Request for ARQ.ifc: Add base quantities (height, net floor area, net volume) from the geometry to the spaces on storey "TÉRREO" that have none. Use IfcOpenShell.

First a look at what the model holds.

```python
import ifcopenshell
import ifcopenshell.util.element
import ifcopenshell.util.unit

model = ifcopenshell.open("ARQ.ifc")
print(model.schema)
for unit_type in ("LENGTHUNIT", "AREAUNIT", "VOLUMEUNIT"):
    print(unit_type, ifcopenshell.util.unit.calculate_unit_scale(model, unit_type))
storey = next(s for s in model.by_type("IfcBuildingStorey") if s.Name == "TÉRREO")
spaces = [e for e in ifcopenshell.util.element.get_decomposition(storey) if e.is_a("IfcSpace")]
for e in sorted(spaces, key=lambda e: e.id()):
    print(e.id(), e.is_a(), e.Name, list(ifcopenshell.util.element.get_psets(e, qtos_only=True)), sep=" | ")
```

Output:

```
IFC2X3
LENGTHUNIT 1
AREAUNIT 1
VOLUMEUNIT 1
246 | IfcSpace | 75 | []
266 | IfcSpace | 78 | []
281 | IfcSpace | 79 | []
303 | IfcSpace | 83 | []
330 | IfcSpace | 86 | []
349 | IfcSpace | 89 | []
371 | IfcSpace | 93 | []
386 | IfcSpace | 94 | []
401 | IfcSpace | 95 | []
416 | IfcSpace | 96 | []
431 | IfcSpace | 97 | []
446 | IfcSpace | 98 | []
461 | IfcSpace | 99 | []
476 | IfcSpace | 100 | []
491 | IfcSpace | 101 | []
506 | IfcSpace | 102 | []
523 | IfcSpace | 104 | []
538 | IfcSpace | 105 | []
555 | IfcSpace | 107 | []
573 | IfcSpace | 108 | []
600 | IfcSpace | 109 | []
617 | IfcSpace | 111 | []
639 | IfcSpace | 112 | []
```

```python
import ifcopenshell
import ifcopenshell.api.pset
import ifcopenshell.geom
import ifcopenshell.util.element
import ifcopenshell.util.shape
import ifcopenshell.util.unit

model = ifcopenshell.open("ARQ.ifc")
unit_scale = ifcopenshell.util.unit.calculate_unit_scale(model)
area_scale = ifcopenshell.util.unit.calculate_unit_scale(model, "AREAUNIT")
volume_scale = ifcopenshell.util.unit.calculate_unit_scale(model, "VOLUMEUNIT")
settings = ifcopenshell.geom.settings()

storey = next(s for s in model.by_type("IfcBuildingStorey") if s.Name == "TÉRREO")
spaces = [e for e in ifcopenshell.util.element.get_decomposition(storey) if e.is_a("IfcSpace")]

for e in sorted(spaces, key=lambda e: e.id()):
    if ifcopenshell.util.element.get_psets(e, qtos_only=True, should_inherit=False):
        continue
    # Geometry comes back in metres, in the element's own axes.
    shape = ifcopenshell.geom.create_shape(settings, e)
    values = {
        "Height": ifcopenshell.util.shape.get_z(shape.geometry) / unit_scale,
        "NetFloorArea": ifcopenshell.util.shape.get_footprint_area(shape.geometry) / area_scale,
        "NetVolume": ifcopenshell.util.shape.get_volume(shape.geometry) / volume_scale,
    }
    qto = ifcopenshell.api.pset.add_qto(model, product=e, name="BaseQuantities")
    ifcopenshell.api.pset.edit_qto(model, qto=qto, properties=values)
    print(e.id(), {k: round(v, 3) for k, v in values.items()})

model.write("ARQ_updated.ifc")
```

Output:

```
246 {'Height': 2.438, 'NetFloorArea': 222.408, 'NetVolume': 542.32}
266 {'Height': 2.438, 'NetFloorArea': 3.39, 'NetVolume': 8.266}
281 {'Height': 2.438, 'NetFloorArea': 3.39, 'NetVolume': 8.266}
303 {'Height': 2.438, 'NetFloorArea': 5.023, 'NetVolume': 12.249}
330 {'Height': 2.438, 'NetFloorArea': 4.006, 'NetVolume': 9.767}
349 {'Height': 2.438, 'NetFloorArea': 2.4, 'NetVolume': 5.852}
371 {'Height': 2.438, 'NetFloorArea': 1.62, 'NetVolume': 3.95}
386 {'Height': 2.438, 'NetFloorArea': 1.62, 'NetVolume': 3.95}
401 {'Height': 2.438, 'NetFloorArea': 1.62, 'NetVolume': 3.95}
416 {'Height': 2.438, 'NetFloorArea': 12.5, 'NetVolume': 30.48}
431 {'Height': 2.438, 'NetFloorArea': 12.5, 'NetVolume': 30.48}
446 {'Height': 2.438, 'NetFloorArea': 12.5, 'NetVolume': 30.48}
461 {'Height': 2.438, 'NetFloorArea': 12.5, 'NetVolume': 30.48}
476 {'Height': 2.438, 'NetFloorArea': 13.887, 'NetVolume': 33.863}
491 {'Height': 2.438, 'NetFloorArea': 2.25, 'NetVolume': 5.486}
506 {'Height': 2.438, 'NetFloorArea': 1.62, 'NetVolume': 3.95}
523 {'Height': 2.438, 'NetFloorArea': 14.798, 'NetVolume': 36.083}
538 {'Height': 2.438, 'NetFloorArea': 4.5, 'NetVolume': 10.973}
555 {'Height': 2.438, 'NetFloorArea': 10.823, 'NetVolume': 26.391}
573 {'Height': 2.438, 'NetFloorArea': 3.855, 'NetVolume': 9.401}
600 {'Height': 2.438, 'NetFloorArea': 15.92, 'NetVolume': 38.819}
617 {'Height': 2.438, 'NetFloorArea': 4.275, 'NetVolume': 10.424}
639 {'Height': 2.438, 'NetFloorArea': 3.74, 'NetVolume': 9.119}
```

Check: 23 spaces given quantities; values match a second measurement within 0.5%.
